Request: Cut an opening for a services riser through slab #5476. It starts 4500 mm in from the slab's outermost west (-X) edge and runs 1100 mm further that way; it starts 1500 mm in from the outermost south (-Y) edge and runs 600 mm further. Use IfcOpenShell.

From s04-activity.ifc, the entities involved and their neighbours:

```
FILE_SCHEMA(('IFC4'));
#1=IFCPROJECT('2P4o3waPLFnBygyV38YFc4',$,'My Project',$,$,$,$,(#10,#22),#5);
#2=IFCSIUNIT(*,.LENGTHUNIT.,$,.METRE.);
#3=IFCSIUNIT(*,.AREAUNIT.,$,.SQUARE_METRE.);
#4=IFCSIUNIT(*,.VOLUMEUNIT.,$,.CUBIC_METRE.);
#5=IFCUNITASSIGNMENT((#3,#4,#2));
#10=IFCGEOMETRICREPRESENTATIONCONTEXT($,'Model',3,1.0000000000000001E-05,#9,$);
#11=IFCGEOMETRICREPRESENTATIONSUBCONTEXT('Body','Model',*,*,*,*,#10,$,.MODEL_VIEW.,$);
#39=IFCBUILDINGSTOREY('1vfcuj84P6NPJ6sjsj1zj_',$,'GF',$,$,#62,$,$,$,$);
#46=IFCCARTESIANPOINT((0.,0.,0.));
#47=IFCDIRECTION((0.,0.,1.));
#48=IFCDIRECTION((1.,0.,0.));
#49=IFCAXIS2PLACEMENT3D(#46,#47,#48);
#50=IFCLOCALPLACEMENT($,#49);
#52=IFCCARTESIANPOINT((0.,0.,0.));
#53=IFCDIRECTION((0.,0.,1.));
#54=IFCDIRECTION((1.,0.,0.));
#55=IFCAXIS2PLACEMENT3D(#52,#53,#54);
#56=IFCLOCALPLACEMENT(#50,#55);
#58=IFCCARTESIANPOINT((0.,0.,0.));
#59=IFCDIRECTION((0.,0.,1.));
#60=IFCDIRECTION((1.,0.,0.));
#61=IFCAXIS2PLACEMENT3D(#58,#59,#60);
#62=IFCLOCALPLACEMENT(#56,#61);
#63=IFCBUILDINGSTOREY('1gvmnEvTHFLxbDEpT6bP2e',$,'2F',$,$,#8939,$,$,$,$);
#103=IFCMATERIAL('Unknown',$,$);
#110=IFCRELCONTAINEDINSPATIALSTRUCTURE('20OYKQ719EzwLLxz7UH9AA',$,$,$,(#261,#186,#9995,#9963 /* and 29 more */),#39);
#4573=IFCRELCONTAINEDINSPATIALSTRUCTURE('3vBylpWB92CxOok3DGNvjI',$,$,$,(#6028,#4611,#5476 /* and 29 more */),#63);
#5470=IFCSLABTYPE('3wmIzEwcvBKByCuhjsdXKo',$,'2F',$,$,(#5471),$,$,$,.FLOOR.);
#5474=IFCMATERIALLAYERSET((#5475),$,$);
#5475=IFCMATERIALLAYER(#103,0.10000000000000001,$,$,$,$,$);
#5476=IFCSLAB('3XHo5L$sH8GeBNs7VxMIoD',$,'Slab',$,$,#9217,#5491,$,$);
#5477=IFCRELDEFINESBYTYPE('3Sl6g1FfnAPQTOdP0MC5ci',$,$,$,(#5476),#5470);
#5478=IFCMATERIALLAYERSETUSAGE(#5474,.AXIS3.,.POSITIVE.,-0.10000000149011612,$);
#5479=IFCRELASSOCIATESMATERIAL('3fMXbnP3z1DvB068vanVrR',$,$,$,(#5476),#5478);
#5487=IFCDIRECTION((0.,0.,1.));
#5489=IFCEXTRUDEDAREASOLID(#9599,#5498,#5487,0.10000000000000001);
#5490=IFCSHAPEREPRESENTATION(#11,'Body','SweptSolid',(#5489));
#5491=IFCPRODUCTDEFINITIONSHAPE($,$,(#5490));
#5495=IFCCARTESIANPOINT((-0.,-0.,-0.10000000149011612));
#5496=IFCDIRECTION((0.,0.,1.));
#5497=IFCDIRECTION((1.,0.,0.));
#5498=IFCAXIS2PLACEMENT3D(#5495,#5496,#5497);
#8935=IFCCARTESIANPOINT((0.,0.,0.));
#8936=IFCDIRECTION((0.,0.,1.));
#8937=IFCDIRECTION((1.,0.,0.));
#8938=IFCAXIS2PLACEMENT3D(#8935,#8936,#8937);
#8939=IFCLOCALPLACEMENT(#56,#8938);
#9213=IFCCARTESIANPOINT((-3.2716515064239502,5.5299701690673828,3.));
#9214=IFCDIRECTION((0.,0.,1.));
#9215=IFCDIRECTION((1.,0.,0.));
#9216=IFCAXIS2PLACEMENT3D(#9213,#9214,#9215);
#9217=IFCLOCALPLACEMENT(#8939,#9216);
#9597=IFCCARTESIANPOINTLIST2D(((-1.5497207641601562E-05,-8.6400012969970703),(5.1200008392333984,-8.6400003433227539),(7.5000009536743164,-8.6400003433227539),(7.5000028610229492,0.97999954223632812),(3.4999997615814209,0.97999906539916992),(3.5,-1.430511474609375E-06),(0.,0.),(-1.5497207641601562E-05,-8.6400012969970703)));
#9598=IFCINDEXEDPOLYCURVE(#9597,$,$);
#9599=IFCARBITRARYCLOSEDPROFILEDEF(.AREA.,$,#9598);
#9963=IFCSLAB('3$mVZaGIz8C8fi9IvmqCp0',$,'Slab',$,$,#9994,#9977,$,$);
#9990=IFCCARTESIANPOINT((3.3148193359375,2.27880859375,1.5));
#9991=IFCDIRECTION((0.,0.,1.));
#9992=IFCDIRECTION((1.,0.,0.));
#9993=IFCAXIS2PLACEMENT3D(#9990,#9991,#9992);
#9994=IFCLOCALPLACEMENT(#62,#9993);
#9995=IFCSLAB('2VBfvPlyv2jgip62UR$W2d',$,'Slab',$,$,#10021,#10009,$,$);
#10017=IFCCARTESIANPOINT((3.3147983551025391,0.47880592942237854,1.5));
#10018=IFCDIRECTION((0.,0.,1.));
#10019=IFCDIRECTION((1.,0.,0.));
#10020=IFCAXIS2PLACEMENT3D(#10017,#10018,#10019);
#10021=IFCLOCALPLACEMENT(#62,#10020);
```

```python
import numpy as np
import ifcopenshell
import ifcopenshell.api.feature
import ifcopenshell.api.geometry
import ifcopenshell.api.root
import ifcopenshell.geom
import ifcopenshell.util.placement
import ifcopenshell.util.representation
import ifcopenshell.util.shape
import ifcopenshell.util.unit

model = ifcopenshell.open("s04-activity.ifc")
unit_scale = ifcopenshell.util.unit.calculate_unit_scale(model)
settings = ifcopenshell.geom.settings()


def volume(element):
    """Net volume in cubic metres, openings subtracted."""
    shape = ifcopenshell.geom.create_shape(settings, element)
    return ifcopenshell.util.shape.get_volume(shape.geometry)


slab = model.by_id(5476)
before = volume(slab)

# Extent in the slab's own axes, in metres. The edges named are its -X and -Y sides.
slab_shape = ifcopenshell.geom.create_shape(settings, slab)
vertices = ifcopenshell.util.shape.get_vertices(slab_shape.geometry)
x_min, y_min, bottom = vertices.min(axis=0)
top = vertices[:, 2].max()

opening = ifcopenshell.api.root.create_entity(model, ifc_class="IfcOpeningElement", name="Services riser opening", predefined_type="OPENING")
context = ifcopenshell.util.representation.get_context(model, "Model", "Body", "MODEL_VIEW")
width, depth = 1.1, 0.6
outline = [(0.0, 0.0), (width, 0.0), (width, depth), (0.0, depth), (0.0, 0.0)]
# Overshoot both faces by 50 mm so the cut is clean.
shape = ifcopenshell.api.geometry.add_slab_representation(
    model, context=context, depth=top - bottom + 0.1, polyline=outline
)
ifcopenshell.api.geometry.assign_representation(model, product=opening, representation=shape)

matrix = ifcopenshell.util.placement.get_local_placement(slab.ObjectPlacement)
matrix[:, 3] = matrix @ np.append(np.array([x_min + 4.5, y_min + 1.5, bottom - 0.05]) / unit_scale, 1.0)
ifcopenshell.api.geometry.edit_object_placement(model, product=opening, matrix=matrix, is_si=False)
ifcopenshell.api.feature.add_feature(model, feature=opening, element=slab)

after = volume(slab)

print(f"slab volume {before:.3f} -> {after:.3f} m3")

model.write("s04-activity-out.ifc")
```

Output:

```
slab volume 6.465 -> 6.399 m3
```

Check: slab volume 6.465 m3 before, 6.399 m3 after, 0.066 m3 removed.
